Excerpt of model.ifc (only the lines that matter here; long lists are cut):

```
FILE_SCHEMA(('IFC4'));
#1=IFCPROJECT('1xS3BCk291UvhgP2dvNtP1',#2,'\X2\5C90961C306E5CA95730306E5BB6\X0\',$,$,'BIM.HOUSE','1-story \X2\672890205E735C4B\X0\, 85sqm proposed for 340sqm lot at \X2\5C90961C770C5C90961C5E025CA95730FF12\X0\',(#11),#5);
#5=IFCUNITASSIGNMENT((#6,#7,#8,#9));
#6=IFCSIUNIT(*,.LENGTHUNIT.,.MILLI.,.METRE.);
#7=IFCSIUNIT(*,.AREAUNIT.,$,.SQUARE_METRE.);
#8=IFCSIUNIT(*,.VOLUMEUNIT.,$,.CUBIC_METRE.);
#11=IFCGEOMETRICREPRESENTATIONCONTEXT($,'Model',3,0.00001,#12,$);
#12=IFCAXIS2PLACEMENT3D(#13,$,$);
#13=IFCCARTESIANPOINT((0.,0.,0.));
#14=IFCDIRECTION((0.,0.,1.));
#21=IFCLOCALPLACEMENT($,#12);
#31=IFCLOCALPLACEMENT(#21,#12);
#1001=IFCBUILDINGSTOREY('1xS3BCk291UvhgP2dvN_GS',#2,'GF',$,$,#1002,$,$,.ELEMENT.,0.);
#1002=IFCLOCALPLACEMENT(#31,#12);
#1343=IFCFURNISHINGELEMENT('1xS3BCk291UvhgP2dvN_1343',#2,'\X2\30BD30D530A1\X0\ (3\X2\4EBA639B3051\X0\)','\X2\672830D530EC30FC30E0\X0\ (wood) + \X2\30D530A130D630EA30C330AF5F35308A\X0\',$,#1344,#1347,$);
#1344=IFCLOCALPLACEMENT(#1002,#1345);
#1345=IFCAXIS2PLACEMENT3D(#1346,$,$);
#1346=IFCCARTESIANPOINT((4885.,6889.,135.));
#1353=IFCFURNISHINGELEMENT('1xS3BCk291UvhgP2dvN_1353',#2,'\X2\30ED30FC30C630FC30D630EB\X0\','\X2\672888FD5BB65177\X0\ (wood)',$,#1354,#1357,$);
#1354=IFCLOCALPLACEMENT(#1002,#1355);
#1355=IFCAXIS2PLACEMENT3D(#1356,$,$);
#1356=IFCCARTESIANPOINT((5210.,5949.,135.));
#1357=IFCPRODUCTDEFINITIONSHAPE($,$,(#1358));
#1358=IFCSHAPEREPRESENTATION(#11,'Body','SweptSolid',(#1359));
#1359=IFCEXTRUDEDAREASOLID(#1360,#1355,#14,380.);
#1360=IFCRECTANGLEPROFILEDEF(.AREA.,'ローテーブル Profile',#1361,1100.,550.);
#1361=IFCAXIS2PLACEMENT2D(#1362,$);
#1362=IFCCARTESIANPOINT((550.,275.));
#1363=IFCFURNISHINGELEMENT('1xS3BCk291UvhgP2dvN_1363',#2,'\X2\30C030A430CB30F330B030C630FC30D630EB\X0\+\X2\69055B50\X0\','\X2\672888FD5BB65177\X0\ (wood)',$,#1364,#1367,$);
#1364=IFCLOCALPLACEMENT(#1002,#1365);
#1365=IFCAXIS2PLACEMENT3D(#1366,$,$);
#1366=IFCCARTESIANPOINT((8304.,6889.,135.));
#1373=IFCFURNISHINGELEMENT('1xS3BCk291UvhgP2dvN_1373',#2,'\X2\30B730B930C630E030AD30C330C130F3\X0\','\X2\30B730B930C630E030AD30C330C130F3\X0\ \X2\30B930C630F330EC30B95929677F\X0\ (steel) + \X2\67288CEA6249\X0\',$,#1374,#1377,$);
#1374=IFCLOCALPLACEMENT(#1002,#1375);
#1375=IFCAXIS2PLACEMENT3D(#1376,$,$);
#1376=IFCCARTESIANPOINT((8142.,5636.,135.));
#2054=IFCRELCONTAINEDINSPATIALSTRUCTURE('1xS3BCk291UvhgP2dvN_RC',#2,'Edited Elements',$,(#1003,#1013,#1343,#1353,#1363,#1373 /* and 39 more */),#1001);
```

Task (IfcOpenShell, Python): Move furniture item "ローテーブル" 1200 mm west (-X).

```python
import ifcopenshell
import ifcopenshell.api.geometry
import ifcopenshell.util.placement

model = ifcopenshell.open("model.ifc")

item = model.by_guid("1xS3BCk291UvhgP2dvN_1353")
matrix = ifcopenshell.util.placement.get_local_placement(item.ObjectPlacement)
matrix[0, 3] -= 1200.0
ifcopenshell.api.geometry.edit_object_placement(model, product=item, matrix=matrix, is_si=False)

print(ifcopenshell.util.placement.get_local_placement(item.ObjectPlacement).round(3) + 0.0)

model.write("model_v2.ifc")
```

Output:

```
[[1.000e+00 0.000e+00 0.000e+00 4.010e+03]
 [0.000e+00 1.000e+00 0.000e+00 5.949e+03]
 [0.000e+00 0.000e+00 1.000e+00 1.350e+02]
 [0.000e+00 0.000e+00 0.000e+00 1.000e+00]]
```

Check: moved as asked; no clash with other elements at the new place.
